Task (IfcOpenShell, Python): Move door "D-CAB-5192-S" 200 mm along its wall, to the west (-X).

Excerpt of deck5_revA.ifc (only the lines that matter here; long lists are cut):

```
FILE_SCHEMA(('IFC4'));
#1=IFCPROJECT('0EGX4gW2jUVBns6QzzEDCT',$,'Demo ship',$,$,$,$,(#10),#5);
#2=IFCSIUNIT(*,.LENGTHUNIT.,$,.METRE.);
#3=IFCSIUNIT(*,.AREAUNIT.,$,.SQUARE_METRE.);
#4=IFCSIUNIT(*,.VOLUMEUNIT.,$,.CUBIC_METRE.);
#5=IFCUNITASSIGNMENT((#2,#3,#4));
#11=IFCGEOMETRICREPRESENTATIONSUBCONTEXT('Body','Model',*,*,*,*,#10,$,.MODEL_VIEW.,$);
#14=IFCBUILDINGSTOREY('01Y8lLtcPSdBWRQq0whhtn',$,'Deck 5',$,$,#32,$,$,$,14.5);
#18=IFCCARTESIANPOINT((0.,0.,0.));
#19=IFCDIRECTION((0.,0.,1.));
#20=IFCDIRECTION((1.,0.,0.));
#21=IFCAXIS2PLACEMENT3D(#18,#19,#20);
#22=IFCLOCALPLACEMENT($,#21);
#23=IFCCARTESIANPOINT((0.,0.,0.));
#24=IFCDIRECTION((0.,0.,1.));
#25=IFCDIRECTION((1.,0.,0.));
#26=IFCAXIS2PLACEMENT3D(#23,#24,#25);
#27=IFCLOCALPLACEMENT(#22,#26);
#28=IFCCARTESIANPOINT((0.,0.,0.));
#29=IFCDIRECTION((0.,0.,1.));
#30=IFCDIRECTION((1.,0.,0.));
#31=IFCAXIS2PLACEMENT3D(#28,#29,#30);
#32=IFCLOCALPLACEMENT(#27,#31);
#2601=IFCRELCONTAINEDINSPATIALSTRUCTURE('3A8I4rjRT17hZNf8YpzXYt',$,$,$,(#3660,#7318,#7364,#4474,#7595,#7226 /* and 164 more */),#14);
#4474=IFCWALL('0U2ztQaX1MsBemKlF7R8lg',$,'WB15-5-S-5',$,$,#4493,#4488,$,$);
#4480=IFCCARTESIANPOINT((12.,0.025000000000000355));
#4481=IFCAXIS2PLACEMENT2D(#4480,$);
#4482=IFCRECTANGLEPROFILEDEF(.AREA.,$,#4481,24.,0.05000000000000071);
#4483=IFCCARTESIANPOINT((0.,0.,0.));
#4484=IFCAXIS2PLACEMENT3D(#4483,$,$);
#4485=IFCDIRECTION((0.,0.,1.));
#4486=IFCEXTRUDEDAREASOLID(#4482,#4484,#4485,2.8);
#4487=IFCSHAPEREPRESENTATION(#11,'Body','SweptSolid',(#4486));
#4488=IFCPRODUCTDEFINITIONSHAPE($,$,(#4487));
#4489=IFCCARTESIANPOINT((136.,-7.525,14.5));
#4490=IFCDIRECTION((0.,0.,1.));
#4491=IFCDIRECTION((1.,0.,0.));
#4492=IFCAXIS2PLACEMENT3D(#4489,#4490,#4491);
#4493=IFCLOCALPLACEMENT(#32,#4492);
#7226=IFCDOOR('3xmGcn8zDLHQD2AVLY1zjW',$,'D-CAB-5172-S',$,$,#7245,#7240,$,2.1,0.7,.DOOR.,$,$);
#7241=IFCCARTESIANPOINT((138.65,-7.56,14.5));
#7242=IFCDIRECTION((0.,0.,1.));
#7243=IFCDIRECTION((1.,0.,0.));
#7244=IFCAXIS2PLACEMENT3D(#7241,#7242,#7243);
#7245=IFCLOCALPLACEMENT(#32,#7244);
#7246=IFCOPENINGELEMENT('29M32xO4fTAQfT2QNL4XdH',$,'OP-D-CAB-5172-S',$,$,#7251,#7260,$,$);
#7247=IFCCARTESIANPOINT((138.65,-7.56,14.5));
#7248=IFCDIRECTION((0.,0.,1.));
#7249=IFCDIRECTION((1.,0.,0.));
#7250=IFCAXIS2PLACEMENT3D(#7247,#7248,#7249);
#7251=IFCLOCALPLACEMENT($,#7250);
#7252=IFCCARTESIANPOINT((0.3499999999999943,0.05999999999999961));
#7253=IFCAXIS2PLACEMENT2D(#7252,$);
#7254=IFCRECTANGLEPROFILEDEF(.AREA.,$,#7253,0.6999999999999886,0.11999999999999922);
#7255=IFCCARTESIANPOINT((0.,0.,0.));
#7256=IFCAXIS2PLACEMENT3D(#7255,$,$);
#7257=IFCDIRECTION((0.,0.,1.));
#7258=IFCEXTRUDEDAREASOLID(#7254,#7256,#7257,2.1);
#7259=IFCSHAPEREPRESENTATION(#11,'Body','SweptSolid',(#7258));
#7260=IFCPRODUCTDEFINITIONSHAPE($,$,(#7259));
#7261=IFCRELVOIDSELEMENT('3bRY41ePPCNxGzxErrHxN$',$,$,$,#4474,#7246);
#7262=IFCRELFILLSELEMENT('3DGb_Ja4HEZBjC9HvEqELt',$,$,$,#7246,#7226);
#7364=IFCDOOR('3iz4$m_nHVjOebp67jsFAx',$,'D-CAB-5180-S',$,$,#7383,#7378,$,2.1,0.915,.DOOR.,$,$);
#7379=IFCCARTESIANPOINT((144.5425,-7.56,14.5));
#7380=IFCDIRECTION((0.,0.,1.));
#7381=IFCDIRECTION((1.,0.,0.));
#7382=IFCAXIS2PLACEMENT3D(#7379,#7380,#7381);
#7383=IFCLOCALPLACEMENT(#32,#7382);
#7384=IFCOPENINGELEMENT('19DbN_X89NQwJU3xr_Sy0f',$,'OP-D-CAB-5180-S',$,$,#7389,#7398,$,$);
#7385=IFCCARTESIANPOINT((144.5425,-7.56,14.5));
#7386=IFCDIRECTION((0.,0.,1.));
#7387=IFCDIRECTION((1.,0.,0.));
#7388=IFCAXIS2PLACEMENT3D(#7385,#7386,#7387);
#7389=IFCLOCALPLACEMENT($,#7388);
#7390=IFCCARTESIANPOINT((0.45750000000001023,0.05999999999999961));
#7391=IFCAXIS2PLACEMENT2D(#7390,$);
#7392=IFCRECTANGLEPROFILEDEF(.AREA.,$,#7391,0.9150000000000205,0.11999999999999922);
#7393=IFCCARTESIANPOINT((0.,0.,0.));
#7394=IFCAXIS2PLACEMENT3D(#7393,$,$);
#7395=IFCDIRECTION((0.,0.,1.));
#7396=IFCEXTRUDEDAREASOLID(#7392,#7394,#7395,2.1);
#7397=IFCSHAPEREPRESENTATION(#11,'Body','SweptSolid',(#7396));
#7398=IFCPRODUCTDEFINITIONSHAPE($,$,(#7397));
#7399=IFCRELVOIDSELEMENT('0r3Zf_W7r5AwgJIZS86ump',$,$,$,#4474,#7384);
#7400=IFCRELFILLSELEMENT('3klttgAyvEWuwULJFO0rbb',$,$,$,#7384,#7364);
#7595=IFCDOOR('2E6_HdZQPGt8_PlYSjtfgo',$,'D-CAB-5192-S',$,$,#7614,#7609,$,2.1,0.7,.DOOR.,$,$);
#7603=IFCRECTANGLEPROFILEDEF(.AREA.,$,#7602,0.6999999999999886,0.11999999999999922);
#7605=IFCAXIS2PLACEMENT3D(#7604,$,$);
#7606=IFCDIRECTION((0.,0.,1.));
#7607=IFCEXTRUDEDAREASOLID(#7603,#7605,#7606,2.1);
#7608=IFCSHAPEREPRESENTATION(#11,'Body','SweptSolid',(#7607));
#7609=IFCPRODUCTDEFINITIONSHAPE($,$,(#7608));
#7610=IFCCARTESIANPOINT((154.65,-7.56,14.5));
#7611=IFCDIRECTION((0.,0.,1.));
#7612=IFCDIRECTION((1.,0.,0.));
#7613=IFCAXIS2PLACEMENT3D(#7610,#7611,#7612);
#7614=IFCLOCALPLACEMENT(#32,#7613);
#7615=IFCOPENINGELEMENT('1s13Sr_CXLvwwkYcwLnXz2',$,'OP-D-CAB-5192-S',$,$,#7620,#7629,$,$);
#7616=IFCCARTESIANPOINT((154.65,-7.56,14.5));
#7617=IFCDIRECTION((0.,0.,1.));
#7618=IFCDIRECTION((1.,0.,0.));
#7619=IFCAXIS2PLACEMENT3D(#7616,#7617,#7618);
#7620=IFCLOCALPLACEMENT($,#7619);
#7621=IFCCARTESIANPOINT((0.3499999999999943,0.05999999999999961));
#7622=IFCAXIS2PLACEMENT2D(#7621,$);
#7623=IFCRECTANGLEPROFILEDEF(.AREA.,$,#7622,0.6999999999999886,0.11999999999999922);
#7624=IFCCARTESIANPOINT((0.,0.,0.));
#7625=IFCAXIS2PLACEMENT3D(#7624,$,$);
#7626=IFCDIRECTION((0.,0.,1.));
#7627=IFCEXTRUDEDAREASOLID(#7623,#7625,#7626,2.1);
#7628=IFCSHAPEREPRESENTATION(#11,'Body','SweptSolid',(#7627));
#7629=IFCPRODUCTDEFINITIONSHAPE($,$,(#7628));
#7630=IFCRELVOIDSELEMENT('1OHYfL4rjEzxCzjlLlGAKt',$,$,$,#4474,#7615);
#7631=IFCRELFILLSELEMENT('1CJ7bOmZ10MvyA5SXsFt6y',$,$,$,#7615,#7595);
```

```python
import ifcopenshell
import ifcopenshell.api.geometry
import ifcopenshell.util.placement

model = ifcopenshell.open("deck5_revA.ifc")

door = model.by_guid("2E6_HdZQPGt8_PlYSjtfgo")
opening = door.FillsVoids[0].RelatingOpeningElement
wall = opening.VoidsElements[0].RelatingBuildingElement

wall_matrix = ifcopenshell.util.placement.get_local_placement(wall.ObjectPlacement)
shift = wall_matrix[:3, 0] * -0.2
before = ifcopenshell.util.placement.get_local_placement(door.ObjectPlacement)[:3, 3].copy()

# The door is not placed relative to its opening, so move both.
for product in (opening, door):
    matrix = ifcopenshell.util.placement.get_local_placement(product.ObjectPlacement)
    matrix[:3, 3] += shift
    ifcopenshell.api.geometry.edit_object_placement(model, product=product, matrix=matrix, is_si=False)

after = ifcopenshell.util.placement.get_local_placement(door.ObjectPlacement)[:3, 3]
print("door moved by", (after - before).round(3) + 0.0)

model.write("deck5_revA_updated.ifc")
```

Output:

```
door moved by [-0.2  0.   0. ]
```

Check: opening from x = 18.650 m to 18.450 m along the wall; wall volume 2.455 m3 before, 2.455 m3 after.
